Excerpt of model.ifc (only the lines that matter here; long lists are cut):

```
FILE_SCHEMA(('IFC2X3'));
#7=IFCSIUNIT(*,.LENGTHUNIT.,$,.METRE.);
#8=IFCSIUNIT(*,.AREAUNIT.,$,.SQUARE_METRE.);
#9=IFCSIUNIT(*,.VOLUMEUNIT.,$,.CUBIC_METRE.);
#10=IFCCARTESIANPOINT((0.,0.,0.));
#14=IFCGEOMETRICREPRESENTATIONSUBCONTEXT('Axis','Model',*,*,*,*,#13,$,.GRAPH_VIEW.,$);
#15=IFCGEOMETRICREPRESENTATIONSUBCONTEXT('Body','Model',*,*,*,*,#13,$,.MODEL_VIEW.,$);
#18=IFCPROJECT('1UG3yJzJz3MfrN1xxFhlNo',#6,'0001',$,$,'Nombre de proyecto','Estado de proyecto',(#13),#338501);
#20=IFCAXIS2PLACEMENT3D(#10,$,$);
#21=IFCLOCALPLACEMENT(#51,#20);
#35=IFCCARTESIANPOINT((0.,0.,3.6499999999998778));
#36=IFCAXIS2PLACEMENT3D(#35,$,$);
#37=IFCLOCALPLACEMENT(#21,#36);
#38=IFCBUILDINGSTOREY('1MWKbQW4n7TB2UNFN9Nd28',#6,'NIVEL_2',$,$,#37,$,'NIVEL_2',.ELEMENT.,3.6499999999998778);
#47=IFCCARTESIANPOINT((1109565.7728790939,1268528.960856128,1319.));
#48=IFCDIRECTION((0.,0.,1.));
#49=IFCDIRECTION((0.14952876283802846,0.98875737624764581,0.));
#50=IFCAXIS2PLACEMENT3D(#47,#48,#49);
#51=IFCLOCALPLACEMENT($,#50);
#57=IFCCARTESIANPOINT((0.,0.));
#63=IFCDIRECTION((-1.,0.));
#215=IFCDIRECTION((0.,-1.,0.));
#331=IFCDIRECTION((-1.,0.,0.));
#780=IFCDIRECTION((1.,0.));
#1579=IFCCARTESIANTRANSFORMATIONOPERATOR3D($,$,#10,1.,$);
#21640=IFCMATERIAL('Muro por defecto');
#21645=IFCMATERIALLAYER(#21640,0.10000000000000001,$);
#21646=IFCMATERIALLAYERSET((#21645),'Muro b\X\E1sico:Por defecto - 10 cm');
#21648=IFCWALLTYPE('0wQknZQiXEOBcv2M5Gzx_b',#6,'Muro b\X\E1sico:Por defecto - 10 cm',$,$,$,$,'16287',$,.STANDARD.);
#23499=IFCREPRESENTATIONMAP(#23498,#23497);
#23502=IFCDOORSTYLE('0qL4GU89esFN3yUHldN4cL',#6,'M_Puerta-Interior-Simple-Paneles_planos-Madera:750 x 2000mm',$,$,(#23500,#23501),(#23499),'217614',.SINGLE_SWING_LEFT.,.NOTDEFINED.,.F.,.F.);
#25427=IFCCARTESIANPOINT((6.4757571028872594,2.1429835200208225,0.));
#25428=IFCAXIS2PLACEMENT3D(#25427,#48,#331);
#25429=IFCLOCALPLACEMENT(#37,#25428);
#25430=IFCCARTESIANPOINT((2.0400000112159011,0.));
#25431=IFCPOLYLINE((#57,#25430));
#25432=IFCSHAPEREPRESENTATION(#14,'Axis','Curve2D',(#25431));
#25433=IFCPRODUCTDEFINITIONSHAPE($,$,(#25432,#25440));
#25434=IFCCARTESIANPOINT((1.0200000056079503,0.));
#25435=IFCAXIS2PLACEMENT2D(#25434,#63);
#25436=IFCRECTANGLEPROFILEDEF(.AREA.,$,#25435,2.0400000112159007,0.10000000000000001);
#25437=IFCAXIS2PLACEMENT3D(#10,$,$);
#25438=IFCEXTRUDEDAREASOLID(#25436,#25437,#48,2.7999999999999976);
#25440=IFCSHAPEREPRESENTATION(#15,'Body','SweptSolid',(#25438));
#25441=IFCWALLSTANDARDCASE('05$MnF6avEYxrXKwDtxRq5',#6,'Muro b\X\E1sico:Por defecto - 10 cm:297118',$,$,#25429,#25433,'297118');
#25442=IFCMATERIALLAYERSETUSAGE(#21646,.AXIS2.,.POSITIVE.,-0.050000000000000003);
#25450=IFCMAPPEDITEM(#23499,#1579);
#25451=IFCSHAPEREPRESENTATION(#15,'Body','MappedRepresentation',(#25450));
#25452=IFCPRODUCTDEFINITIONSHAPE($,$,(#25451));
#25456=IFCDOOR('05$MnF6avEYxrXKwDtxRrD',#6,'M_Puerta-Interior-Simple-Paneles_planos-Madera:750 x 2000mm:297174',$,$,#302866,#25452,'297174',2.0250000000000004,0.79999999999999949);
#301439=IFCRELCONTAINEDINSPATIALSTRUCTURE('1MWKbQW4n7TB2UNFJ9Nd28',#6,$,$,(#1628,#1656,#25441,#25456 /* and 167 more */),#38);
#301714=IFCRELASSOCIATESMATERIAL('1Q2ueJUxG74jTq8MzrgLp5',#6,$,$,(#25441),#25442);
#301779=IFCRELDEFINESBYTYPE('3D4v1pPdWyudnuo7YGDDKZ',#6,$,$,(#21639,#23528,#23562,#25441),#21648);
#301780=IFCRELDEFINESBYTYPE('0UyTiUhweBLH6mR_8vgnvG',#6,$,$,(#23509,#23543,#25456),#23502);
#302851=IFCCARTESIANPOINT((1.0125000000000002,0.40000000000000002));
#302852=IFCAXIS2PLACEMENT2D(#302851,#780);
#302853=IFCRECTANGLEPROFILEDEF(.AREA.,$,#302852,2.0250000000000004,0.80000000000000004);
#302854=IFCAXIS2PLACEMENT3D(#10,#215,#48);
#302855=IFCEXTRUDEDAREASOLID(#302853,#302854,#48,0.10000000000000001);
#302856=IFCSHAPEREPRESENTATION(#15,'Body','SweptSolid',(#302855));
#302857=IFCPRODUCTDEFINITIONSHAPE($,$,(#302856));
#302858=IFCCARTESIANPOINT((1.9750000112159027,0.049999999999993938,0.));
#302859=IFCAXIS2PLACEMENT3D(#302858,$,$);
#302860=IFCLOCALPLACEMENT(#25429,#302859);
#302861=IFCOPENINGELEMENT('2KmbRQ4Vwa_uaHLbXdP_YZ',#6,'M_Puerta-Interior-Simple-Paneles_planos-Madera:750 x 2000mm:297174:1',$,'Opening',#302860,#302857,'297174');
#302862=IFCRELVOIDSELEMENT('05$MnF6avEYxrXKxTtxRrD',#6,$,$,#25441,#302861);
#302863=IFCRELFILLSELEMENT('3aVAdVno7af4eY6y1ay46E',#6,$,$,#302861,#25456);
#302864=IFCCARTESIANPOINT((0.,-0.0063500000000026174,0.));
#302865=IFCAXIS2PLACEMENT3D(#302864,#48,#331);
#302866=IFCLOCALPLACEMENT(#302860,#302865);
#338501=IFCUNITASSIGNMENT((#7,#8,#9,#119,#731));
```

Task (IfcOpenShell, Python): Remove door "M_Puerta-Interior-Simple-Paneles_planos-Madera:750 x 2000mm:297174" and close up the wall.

```python
import ifcopenshell
import ifcopenshell.api.feature
import ifcopenshell.api.root
import ifcopenshell.geom
import ifcopenshell.util.shape

model = ifcopenshell.open("model.ifc")
settings = ifcopenshell.geom.settings()


def volume(element):
    """Net volume in cubic metres, openings subtracted."""
    shape = ifcopenshell.geom.create_shape(settings, element)
    return ifcopenshell.util.shape.get_volume(shape.geometry)


door = model.by_guid("05$MnF6avEYxrXKwDtxRrD")
opening = door.FillsVoids[0].RelatingOpeningElement
wall = opening.VoidsElements[0].RelatingBuildingElement
before = volume(wall)

ifcopenshell.api.root.remove_product(model, product=door)
ifcopenshell.api.feature.remove_feature(model, feature=opening)

after = volume(wall)

print(f"wall volume {before:.3f} -> {after:.3f} m3")

model.write("model-out.ifc")
```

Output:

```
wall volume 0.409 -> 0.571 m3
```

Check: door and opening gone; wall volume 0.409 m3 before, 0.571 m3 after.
